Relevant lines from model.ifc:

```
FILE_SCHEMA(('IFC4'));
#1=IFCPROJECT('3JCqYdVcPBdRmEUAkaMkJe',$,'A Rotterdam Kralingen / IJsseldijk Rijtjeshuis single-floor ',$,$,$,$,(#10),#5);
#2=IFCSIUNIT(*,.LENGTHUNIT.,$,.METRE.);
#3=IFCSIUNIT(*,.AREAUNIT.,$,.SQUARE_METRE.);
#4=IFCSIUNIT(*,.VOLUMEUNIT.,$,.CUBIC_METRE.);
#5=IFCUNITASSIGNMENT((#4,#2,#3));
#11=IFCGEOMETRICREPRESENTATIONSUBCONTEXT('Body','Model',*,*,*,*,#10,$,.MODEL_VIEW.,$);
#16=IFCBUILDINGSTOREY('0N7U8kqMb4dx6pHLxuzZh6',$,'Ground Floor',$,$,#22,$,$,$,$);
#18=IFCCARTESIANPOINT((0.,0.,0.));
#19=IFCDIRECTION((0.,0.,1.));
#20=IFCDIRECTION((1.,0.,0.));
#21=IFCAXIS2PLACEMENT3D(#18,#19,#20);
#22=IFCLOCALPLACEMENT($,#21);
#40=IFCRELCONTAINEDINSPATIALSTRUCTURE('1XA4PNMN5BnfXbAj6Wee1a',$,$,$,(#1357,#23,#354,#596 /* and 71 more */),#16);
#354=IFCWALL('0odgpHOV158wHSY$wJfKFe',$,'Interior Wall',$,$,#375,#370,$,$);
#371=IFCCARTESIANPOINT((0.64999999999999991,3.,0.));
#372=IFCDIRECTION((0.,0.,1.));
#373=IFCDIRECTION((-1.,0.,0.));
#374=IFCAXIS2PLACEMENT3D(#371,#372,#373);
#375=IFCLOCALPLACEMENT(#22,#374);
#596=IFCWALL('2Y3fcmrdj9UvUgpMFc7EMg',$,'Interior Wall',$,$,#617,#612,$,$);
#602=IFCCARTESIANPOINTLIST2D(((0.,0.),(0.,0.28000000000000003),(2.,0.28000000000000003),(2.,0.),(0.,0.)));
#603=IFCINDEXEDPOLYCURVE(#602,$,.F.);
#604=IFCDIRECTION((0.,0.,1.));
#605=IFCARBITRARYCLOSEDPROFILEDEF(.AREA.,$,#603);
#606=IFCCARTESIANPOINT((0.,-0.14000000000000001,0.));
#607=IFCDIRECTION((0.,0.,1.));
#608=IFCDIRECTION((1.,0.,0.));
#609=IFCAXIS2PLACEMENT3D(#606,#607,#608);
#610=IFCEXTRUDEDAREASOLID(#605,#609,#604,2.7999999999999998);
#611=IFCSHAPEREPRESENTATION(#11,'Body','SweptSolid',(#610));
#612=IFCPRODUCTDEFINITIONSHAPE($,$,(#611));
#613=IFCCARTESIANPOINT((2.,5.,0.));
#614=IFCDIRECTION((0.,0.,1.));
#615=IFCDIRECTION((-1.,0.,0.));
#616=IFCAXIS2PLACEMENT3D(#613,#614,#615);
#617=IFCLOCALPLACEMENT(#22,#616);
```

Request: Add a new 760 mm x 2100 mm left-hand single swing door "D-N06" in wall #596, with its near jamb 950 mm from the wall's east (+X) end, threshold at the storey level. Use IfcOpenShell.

```python
import numpy as np
import ifcopenshell
import ifcopenshell.api.feature
import ifcopenshell.api.geometry
import ifcopenshell.api.root
import ifcopenshell.api.spatial
import ifcopenshell.geom
import ifcopenshell.util.element
import ifcopenshell.util.placement
import ifcopenshell.util.representation
import ifcopenshell.util.shape
import ifcopenshell.util.unit

model = ifcopenshell.open("model.ifc")
unit_scale = ifcopenshell.util.unit.calculate_unit_scale(model)
settings = ifcopenshell.geom.settings()


def volume(element):
    """Net volume in cubic metres, openings subtracted."""
    shape = ifcopenshell.geom.create_shape(settings, element)
    return ifcopenshell.util.shape.get_volume(shape.geometry)


wall = model.by_guid("2Y3fcmrdj9UvUgpMFc7EMg")
storey = ifcopenshell.util.element.get_container(wall, ifc_class="IfcBuildingStorey")
context = ifcopenshell.util.representation.get_context(model, "Model", "Body", "MODEL_VIEW")
before = volume(wall)

width, height, from_end, sill = 0.76, 2.1, 0.95, 0.0  # metres

# The wall runs along its own X axis, and the end named is its -X end.
wall_shape = ifcopenshell.geom.create_shape(settings, wall)
x, y, z = ifcopenshell.util.shape.get_vertices(wall_shape.geometry).T
start = x.min() + from_end
face, thickness = float(y.min()), float(y.max() - y.min())
wall_matrix = ifcopenshell.util.placement.get_local_placement(wall.ObjectPlacement)
level = ifcopenshell.util.placement.get_local_placement(storey.ObjectPlacement)[2, 3]


def in_wall(x, y):
    """Placement at x, y metres in the wall's axes, at sill height."""
    matrix = wall_matrix.copy()
    matrix[:, 3] = wall_matrix @ np.array([x / unit_scale, y / unit_scale, 0.0, 1.0])
    matrix[2, 3] = level + sill / unit_scale
    return matrix


# Opening: a box that overshoots both wall faces by 50 mm.
opening = ifcopenshell.api.root.create_entity(model, ifc_class="IfcOpeningElement", predefined_type="OPENING")
box = ifcopenshell.api.geometry.add_wall_representation(
    model, context=context, length=width, height=height, thickness=thickness + 0.1
)
ifcopenshell.api.geometry.assign_representation(model, product=opening, representation=box)
ifcopenshell.api.geometry.edit_object_placement(model, product=opening, matrix=in_wall(start, face - 0.05), is_si=False)
ifcopenshell.api.feature.add_feature(model, feature=opening, element=wall)

door = ifcopenshell.api.root.create_entity(model, ifc_class="IfcDoor", name="D-N06", predefined_type="DOOR")
door.OverallWidth, door.OverallHeight = width / unit_scale, height / unit_scale
door.OperationType = "SINGLE_SWING_LEFT"
body = ifcopenshell.api.geometry.add_door_representation(
    model,
    context=context,
    overall_width=door.OverallWidth,
    overall_height=door.OverallHeight,
    operation_type="SINGLE_SWING_LEFT",
    lining_properties={"LiningDepth": thickness / unit_scale, "ThresholdDepth": thickness / unit_scale},
)
ifcopenshell.api.geometry.assign_representation(model, product=door, representation=body)
ifcopenshell.api.spatial.assign_container(model, products=[door], relating_structure=storey)
ifcopenshell.api.feature.add_filling(model, opening=opening, element=door)

# The lining spans the wall, so the door starts at the wall face.
ifcopenshell.api.geometry.edit_object_placement(model, product=door, matrix=in_wall(start, face), is_si=False)

after = volume(wall)

print(f"wall volume {before:.3f} -> {after:.3f} m3")

model.write("model_updated.ifc")
```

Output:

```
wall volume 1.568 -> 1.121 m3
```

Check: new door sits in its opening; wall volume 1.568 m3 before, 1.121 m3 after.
